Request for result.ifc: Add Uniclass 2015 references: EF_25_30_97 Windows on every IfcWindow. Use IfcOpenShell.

First a look at what the model holds.

```python
import ifcopenshell

model = ifcopenshell.open("result.ifc")
print(model.schema)
print("classifications:", [c.Name for c in model.by_type("IfcClassification")])
for ifc_class in ("IfcDoor", "IfcRoof", "IfcStair", "IfcWall", "IfcWindow"):
    print(ifc_class, len(model.by_type(ifc_class)))
```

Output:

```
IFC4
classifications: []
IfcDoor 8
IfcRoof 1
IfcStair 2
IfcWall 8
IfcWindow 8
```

```python
import ifcopenshell
import ifcopenshell.api.classification

model = ifcopenshell.open("result.ifc")

system = ifcopenshell.api.classification.add_classification(model, classification="Uniclass 2015")

codes = {
    "IfcWindow": ("EF_25_30_97", "Windows"),
}
for ifc_class, (code, name) in codes.items():
    products = model.by_type(ifc_class)
    ifcopenshell.api.classification.add_reference(
        model, products=products, classification=system, identification=code, name=name
    )
    print(code, len(products))

model.write("result_v2.ifc")
```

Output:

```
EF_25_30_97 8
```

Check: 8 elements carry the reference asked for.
